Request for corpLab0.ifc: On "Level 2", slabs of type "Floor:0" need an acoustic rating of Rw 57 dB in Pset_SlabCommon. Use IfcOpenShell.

First a look at what the model holds.

```python
import ifcopenshell
import ifcopenshell.util.element

model = ifcopenshell.open("corpLab0.ifc")
print(model.schema)
storey = next(s for s in model.by_type("IfcBuildingStorey") if s.Name == "Level 2")
slabs = [e for e in ifcopenshell.util.element.get_decomposition(storey) if e.is_a("IfcSlab")]
seen = {}
for e in slabs:
    element_type = ifcopenshell.util.element.get_type(e)
    key = (element_type.Name if element_type != e and element_type else None, ifcopenshell.util.element.get_pset(e, "Pset_SlabCommon", "AcousticRating"))
    seen[key] = seen.get(key, 0) + 1
for (name, value), count in sorted(seen.items(), key=str):
    print(count, "x", name, "|", value)
```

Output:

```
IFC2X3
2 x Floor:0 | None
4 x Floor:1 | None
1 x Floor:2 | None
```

```python
import ifcopenshell
import ifcopenshell.api.pset
import ifcopenshell.util.element

model = ifcopenshell.open("corpLab0.ifc")

storey = next(s for s in model.by_type("IfcBuildingStorey") if s.Name == "Level 2")
slabs = [e for e in ifcopenshell.util.element.get_decomposition(storey) if e.is_a("IfcSlab")]

count = 0
for e in slabs:
    element_type = ifcopenshell.util.element.get_type(e)
    if element_type in (None, e) or element_type.Name != "Floor:0":
        continue
    # add_pset returns the element's existing set when there is one.
    pset = ifcopenshell.api.pset.add_pset(model, product=e, name="Pset_SlabCommon")
    ifcopenshell.api.pset.edit_pset(model, pset=pset, properties={"AcousticRating": "Rw 57 dB"})
    count += 1

print(count, "slabs updated")

model.write("corpLab0_v2.ifc")
```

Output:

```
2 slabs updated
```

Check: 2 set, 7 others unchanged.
